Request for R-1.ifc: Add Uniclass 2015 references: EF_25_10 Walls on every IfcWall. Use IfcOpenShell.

First a look at what the model holds.

```python
import ifcopenshell

model = ifcopenshell.open("R-1.ifc")
print(model.schema)
print("classifications:", [c.Name for c in model.by_type("IfcClassification")])
for ifc_class in ("IfcDoor", "IfcRoof", "IfcStair", "IfcWall", "IfcWindow"):
    print(ifc_class, len(model.by_type(ifc_class)))
```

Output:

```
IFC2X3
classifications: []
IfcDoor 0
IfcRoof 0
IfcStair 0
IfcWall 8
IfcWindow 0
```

```python
import ifcopenshell
import ifcopenshell.api.classification

model = ifcopenshell.open("R-1.ifc")

# IFC2X3 requires Source and Edition and has no link from the project to the system.
system = model.create_entity("IfcClassification", Source="NBS", Edition="2015", Name="Uniclass 2015")

codes = {
    "IfcWall": ("EF_25_10", "Walls"),
}
for ifc_class, (code, name) in codes.items():
    products = model.by_type(ifc_class)
    ifcopenshell.api.classification.add_reference(
        model, products=products, classification=system, identification=code, name=name
    )
    print(code, len(products))

model.write("R-1_updated.ifc")
```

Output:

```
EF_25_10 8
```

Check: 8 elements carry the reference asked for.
